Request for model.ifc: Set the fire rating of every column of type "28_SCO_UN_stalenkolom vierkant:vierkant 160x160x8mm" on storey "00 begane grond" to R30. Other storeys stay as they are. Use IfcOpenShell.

First a look at what the model holds.

```python
import ifcopenshell
import ifcopenshell.util.element

model = ifcopenshell.open("model.ifc")
print(model.schema)
storey = next(s for s in model.by_type("IfcBuildingStorey") if s.Name == "00 begane grond")
columns = [e for e in ifcopenshell.util.element.get_decomposition(storey) if e.is_a("IfcColumn")]
seen = {}
for e in columns:
    element_type = ifcopenshell.util.element.get_type(e)
    key = (element_type.Name if element_type != e and element_type else None, ifcopenshell.util.element.get_pset(e, "Pset_ColumnCommon", "FireRating"))
    seen[key] = seen.get(key, 0) + 1
for (name, value), count in sorted(seen.items(), key=str):
    print(count, "x", name, "|", value)
```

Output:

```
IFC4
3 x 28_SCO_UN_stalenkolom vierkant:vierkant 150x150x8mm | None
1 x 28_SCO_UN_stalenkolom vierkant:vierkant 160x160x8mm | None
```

```python
import ifcopenshell
import ifcopenshell.api.pset
import ifcopenshell.util.element

model = ifcopenshell.open("model.ifc")

storey = next(s for s in model.by_type("IfcBuildingStorey") if s.Name == "00 begane grond")
columns = [e for e in ifcopenshell.util.element.get_decomposition(storey) if e.is_a("IfcColumn")]

count = 0
for e in columns:
    element_type = ifcopenshell.util.element.get_type(e)
    if element_type in (None, e) or element_type.Name != "28_SCO_UN_stalenkolom vierkant:vierkant 160x160x8mm":
        continue
    # add_pset returns the element's existing set when there is one.
    pset = ifcopenshell.api.pset.add_pset(model, product=e, name="Pset_ColumnCommon")
    ifcopenshell.api.pset.edit_pset(model, pset=pset, properties={"FireRating": "R30"})
    count += 1

print(count, "columns updated")

model.write("model-out.ifc")
```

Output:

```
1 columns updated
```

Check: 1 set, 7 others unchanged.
